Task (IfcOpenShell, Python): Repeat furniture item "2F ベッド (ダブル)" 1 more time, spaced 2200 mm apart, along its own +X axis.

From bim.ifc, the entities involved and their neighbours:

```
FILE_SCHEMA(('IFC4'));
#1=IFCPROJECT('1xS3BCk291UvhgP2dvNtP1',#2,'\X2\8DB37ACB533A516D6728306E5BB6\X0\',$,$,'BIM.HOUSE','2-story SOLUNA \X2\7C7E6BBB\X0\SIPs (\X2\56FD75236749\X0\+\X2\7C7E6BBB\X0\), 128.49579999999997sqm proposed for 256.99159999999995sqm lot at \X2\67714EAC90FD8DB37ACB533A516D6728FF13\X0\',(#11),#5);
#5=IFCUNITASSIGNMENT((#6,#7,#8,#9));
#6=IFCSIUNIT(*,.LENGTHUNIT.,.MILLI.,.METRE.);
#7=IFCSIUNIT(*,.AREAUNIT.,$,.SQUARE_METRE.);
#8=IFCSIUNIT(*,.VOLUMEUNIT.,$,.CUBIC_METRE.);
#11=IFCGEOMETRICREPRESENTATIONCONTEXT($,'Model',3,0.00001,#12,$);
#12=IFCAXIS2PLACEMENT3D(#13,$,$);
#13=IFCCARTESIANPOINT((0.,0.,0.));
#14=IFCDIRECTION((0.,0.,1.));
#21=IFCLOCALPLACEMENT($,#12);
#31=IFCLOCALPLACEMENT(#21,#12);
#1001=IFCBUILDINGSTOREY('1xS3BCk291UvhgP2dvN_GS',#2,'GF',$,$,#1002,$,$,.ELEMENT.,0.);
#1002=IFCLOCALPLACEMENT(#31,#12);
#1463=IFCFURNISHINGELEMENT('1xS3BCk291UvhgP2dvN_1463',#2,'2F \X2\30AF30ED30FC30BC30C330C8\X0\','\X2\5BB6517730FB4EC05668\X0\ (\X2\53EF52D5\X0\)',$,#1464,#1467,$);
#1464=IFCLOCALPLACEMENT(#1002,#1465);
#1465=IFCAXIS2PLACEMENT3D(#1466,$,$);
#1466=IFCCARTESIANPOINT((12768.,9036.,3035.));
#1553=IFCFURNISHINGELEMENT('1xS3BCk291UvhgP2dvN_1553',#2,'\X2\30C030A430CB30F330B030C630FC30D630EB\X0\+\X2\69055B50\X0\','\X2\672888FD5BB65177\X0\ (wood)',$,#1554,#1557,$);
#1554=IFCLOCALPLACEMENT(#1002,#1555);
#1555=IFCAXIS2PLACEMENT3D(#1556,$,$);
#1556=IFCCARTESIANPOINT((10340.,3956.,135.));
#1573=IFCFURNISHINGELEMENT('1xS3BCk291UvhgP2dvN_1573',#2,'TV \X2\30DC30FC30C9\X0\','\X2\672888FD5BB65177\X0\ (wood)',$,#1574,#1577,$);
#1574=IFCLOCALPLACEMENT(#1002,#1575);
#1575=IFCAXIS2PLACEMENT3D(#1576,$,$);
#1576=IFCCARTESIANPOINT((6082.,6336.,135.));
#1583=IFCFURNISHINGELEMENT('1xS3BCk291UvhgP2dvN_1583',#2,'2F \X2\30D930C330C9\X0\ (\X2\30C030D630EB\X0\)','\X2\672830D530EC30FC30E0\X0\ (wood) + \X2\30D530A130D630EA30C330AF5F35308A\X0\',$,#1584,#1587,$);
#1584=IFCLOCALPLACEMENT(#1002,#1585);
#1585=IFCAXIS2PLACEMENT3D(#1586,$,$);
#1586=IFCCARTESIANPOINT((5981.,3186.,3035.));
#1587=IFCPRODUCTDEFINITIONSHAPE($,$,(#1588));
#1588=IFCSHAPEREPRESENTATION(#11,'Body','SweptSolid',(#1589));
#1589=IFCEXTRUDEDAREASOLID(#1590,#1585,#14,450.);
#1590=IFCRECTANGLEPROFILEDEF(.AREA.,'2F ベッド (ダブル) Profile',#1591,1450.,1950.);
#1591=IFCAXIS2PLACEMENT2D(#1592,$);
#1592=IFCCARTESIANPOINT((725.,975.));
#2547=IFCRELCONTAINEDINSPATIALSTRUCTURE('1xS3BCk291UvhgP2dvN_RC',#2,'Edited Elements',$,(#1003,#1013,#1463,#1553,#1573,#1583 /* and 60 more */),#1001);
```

```python
import ifcopenshell
import ifcopenshell.api.geometry
import ifcopenshell.api.root
import ifcopenshell.util.element
import ifcopenshell.util.placement

model = ifcopenshell.open("bim.ifc")


def reuse_history(source, copy):
    """copy_class also copies each property set's owner history, people and application; keep the originals."""
    for rel in copy.IsDefinedBy:
        if rel.is_a("IfcRelDefinesByProperties") and (history := rel.RelatingPropertyDefinition.OwnerHistory):
            rel.RelatingPropertyDefinition.OwnerHistory = source.OwnerHistory
            ifcopenshell.util.element.remove_deep2(model, history)


source = model.by_guid("1xS3BCk291UvhgP2dvN_1583")
base = ifcopenshell.util.placement.get_local_placement(source.ObjectPlacement)
step = base[:3, 0] * 2200.0

for i in range(1, 2):
    copy = ifcopenshell.api.root.copy_class(model, product=source)
    copy.Representation = ifcopenshell.util.element.copy_deep(
        model, source.Representation, exclude=["IfcGeometricRepresentationContext", "IfcRepresentationMap"]
    )
    reuse_history(source, copy)
    matrix = base.copy()
    matrix[:3, 3] += i * step
    print("added at", matrix[:3, 3].round(3) + 0.0)
    ifcopenshell.api.geometry.edit_object_placement(model, product=copy, matrix=matrix, is_si=False)

model.write("bim_v2.ifc")
```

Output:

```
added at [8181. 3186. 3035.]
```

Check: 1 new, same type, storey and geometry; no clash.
